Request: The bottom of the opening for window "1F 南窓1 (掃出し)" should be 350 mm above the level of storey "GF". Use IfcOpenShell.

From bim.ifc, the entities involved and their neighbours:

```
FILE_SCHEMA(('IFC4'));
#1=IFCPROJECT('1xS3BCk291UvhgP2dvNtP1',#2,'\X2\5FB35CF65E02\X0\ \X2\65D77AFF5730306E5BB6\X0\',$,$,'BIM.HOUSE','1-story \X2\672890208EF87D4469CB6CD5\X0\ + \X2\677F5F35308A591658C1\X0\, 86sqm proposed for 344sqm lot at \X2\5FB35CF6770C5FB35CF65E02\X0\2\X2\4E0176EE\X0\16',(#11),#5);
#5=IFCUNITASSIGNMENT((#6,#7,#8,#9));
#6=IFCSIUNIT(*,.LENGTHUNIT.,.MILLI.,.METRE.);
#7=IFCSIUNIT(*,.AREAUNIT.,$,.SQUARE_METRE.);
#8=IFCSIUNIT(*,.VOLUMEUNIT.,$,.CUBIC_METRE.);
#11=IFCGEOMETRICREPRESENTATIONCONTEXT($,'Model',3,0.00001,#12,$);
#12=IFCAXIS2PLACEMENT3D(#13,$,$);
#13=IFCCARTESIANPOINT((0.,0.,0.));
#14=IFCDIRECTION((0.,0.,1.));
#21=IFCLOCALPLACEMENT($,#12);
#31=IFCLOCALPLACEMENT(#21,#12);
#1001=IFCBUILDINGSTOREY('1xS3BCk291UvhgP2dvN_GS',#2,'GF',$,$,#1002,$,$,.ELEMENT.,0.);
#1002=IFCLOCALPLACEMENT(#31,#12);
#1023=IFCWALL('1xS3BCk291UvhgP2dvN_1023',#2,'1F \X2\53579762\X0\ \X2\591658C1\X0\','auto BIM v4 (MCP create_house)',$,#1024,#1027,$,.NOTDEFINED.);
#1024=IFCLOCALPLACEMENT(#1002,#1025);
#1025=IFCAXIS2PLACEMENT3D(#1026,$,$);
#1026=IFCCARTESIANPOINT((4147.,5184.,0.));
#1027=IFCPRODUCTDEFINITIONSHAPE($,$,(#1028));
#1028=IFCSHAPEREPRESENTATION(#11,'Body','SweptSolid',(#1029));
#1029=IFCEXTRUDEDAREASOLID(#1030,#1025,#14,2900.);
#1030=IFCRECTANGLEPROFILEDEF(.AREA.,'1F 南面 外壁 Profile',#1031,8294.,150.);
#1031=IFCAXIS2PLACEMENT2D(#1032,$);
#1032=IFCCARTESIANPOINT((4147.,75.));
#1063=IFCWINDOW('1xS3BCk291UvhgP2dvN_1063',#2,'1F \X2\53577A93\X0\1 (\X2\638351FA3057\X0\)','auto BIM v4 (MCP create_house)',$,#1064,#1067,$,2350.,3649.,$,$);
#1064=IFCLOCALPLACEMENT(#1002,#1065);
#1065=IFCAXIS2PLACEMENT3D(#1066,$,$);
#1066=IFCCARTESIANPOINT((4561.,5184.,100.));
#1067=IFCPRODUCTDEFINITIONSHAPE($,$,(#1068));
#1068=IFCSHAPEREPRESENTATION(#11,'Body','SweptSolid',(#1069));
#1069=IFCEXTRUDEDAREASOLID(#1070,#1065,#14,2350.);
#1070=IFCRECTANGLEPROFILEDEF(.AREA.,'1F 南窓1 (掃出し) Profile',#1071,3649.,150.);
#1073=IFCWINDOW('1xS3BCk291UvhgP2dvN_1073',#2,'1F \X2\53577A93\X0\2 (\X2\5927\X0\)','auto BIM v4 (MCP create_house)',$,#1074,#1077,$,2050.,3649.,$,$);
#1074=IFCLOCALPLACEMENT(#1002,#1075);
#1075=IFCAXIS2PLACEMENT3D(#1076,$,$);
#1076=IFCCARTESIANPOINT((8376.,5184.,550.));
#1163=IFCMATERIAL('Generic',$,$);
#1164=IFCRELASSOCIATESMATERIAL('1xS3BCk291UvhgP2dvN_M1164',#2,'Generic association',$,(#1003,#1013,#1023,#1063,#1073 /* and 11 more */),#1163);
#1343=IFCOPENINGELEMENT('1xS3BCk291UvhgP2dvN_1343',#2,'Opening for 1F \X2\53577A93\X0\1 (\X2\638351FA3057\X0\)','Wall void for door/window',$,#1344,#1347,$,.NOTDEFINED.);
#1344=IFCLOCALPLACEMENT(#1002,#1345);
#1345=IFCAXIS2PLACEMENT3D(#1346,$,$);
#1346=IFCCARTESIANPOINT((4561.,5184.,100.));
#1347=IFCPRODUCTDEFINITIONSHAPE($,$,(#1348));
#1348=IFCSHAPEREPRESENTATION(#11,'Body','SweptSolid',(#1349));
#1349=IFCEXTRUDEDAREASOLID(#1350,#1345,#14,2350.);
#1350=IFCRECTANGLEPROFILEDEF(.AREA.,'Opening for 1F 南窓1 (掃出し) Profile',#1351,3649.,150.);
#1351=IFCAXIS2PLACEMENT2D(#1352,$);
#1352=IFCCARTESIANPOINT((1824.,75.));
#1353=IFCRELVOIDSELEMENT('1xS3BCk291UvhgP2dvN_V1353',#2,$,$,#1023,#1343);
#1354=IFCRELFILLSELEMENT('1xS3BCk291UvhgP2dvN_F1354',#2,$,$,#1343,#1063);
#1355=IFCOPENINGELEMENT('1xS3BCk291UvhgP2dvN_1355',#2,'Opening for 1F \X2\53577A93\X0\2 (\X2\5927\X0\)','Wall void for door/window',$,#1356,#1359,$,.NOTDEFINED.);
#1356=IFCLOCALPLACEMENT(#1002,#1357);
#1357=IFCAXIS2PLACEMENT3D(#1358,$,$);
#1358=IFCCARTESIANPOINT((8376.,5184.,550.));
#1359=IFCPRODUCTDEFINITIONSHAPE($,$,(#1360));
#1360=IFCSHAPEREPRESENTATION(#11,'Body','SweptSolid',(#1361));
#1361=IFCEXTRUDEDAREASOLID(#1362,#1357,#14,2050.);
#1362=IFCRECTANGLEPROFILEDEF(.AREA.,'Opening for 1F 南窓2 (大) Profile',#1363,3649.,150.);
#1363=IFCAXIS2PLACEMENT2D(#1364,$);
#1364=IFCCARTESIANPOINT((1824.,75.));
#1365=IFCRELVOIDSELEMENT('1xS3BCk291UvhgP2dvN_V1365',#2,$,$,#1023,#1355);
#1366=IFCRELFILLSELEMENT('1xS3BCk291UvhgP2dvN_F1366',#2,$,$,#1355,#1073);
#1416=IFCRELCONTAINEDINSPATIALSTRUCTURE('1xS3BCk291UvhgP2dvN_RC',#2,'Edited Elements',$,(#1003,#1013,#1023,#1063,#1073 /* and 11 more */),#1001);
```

```python
import numpy as np
import ifcopenshell
import ifcopenshell.api.geometry
import ifcopenshell.geom
import ifcopenshell.util.element
import ifcopenshell.util.placement
import ifcopenshell.util.shape
import ifcopenshell.util.unit

model = ifcopenshell.open("bim.ifc")
unit_scale = ifcopenshell.util.unit.calculate_unit_scale(model)

window = model.by_guid("1xS3BCk291UvhgP2dvN_1063")
opening = window.FillsVoids[0].RelatingOpeningElement
storey = ifcopenshell.util.element.get_container(window, ifc_class="IfcBuildingStorey")
level = ifcopenshell.util.placement.get_local_placement(storey.ObjectPlacement)[2, 3]

# The opening's origin need not be at the sill, so measure its lowest point.
shape = ifcopenshell.geom.create_shape(ifcopenshell.geom.settings(), opening)
bottom = ifcopenshell.util.shape.get_shape_bottom_elevation(shape, shape.geometry) / unit_scale
dz = level + 0.35 / unit_scale - bottom

shift = np.array([0.0, 0.0, dz])
# The window is not placed relative to its opening, so move both.
for product in (opening, window):
    matrix = ifcopenshell.util.placement.get_local_placement(product.ObjectPlacement)
    matrix[:3, 3] += shift
    ifcopenshell.api.geometry.edit_object_placement(model, product=product, matrix=matrix, is_si=False)

print(f"moved by {dz * unit_scale:+.3f} m")

model.write("bim_edited.ifc")
```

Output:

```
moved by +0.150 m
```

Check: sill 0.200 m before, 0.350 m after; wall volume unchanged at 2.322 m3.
